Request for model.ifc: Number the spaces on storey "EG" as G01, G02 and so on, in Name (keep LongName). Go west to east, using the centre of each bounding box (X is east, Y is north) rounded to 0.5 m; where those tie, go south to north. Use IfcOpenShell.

First a look at what the model holds.

```python
import ifcopenshell
import ifcopenshell.util.element
import ifcopenshell.util.placement

model = ifcopenshell.open("model.ifc")
print(model.schema)
storey = next(s for s in model.by_type("IfcBuildingStorey") if s.Name == "EG")
spaces = [e for e in ifcopenshell.util.element.get_decomposition(storey) if e.is_a("IfcSpace")]
for e in sorted(spaces, key=lambda e: e.id()):
    origin = ifcopenshell.util.placement.get_local_placement(e.ObjectPlacement)[:3, 3]
    print(e.id(), e.Name, e.LongName, origin.round(2) + 0.0, sep=" | ")
```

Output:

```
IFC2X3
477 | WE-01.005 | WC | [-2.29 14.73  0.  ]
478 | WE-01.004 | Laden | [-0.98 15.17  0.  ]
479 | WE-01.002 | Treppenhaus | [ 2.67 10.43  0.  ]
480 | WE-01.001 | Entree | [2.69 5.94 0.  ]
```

```python
import ifcopenshell
import ifcopenshell.geom
import ifcopenshell.util.element
import ifcopenshell.util.shape

model = ifcopenshell.open("model.ifc")
settings = ifcopenshell.geom.settings()
settings.set("use-world-coords", True)


def centre(element):
    shape = ifcopenshell.geom.create_shape(settings, element)
    return ifcopenshell.util.shape.get_bbox_centroid(shape.geometry)


storey = next(s for s in model.by_type("IfcBuildingStorey") if s.Name == "EG")
spaces = [e for e in ifcopenshell.util.element.get_decomposition(storey) if e.is_a("IfcSpace")]

# Insertion points can sit at a corner or the storey origin, so sort by the geometry (in metres).
centres = {e: centre(e) for e in spaces}
spaces.sort(key=lambda e: (round(centres[e][0] / 0.5), centres[e][1]))

for i, e in enumerate(spaces, start=1):
    number = f"G{i:02d}"
    e.Name = number
    print(e.id(), number)

model.write("model_rev.ifc")
```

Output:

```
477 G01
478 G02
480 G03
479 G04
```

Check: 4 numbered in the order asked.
